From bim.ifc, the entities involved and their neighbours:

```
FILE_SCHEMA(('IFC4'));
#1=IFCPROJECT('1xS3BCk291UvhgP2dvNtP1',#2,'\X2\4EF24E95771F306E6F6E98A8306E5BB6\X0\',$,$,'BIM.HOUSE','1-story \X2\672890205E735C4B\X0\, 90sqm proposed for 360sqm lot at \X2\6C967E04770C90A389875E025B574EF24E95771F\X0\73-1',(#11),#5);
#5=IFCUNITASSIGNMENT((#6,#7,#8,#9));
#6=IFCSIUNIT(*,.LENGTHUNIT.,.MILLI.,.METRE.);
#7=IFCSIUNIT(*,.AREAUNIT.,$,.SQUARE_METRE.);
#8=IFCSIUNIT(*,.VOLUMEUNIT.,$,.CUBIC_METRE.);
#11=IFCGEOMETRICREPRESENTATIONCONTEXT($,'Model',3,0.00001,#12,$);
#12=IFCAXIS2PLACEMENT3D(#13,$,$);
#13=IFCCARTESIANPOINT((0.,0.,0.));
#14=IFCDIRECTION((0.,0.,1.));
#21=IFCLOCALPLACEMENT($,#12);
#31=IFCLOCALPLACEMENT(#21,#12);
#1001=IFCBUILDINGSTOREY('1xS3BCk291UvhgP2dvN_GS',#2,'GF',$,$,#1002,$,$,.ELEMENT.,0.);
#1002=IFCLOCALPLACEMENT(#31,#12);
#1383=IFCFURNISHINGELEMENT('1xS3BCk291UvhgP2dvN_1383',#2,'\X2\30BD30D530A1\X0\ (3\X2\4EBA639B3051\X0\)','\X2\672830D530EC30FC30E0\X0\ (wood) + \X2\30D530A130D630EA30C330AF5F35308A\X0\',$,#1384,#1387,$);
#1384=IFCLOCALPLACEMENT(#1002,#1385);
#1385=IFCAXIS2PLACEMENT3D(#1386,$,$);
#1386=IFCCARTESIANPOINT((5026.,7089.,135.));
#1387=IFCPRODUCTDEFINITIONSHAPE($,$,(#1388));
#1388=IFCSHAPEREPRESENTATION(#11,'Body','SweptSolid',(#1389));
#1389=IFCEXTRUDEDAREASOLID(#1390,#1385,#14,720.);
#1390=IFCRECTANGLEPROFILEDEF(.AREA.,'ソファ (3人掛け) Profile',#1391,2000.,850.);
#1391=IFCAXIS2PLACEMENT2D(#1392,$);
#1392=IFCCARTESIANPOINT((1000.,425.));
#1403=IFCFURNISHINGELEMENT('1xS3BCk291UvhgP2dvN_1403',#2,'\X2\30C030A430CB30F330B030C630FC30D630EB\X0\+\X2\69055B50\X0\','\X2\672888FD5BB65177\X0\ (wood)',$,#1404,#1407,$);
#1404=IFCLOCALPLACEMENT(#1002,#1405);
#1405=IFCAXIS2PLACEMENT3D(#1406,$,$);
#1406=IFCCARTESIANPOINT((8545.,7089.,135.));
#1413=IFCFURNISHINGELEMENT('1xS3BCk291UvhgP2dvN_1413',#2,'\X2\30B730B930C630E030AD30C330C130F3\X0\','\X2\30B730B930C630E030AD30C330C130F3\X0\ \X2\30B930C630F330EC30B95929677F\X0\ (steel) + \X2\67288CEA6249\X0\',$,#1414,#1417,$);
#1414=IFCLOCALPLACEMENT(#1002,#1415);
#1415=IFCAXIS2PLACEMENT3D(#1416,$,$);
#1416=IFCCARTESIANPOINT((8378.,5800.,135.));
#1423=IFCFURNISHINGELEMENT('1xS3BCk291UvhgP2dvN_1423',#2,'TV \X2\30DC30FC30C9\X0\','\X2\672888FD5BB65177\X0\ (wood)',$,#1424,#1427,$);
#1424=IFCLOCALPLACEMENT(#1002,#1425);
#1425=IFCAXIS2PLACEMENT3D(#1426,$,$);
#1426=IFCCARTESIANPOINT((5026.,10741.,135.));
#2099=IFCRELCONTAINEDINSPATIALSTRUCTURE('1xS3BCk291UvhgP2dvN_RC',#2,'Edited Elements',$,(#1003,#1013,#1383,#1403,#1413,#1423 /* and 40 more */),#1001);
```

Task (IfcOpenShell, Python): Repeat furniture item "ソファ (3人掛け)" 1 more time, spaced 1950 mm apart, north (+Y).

```python
import numpy as np
import ifcopenshell
import ifcopenshell.api.geometry
import ifcopenshell.api.root
import ifcopenshell.util.element
import ifcopenshell.util.placement

model = ifcopenshell.open("bim.ifc")


def reuse_history(source, copy):
    """copy_class also copies each property set's owner history, people and application; keep the originals."""
    for rel in copy.IsDefinedBy:
        if rel.is_a("IfcRelDefinesByProperties") and (history := rel.RelatingPropertyDefinition.OwnerHistory):
            rel.RelatingPropertyDefinition.OwnerHistory = source.OwnerHistory
            ifcopenshell.util.element.remove_deep2(model, history)


source = model.by_id(1383)
base = ifcopenshell.util.placement.get_local_placement(source.ObjectPlacement)
step = np.array([0.0, 1.0, 0.0]) * 1950.0

for i in range(1, 2):
    copy = ifcopenshell.api.root.copy_class(model, product=source)
    copy.Representation = ifcopenshell.util.element.copy_deep(
        model, source.Representation, exclude=["IfcGeometricRepresentationContext", "IfcRepresentationMap"]
    )
    reuse_history(source, copy)
    matrix = base.copy()
    matrix[:3, 3] += i * step
    print("added at", matrix[:3, 3].round(3) + 0.0)
    ifcopenshell.api.geometry.edit_object_placement(model, product=copy, matrix=matrix, is_si=False)

model.write("bim_edited.ifc")
```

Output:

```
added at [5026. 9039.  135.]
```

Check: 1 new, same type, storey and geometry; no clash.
